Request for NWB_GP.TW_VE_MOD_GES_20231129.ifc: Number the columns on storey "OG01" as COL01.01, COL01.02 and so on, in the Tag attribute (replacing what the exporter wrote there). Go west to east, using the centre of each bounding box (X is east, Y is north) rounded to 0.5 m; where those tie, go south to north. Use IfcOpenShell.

First a look at what the model holds.

```python
import ifcopenshell
import ifcopenshell.util.element
import ifcopenshell.util.placement

model = ifcopenshell.open("NWB_GP.TW_VE_MOD_GES_20231129.ifc")
print(model.schema)
storey = next(s for s in model.by_type("IfcBuildingStorey") if s.Name == "OG01")
columns = [e for e in ifcopenshell.util.element.get_decomposition(storey) if e.is_a("IfcColumn")]
for e in sorted(columns, key=lambda e: e.id()):
    origin = ifcopenshell.util.placement.get_local_placement(e.ObjectPlacement)[:3, 3]
    print(e.id(), e.Tag, e.Name, origin.round(2) + 0.0, sep=" | ")
```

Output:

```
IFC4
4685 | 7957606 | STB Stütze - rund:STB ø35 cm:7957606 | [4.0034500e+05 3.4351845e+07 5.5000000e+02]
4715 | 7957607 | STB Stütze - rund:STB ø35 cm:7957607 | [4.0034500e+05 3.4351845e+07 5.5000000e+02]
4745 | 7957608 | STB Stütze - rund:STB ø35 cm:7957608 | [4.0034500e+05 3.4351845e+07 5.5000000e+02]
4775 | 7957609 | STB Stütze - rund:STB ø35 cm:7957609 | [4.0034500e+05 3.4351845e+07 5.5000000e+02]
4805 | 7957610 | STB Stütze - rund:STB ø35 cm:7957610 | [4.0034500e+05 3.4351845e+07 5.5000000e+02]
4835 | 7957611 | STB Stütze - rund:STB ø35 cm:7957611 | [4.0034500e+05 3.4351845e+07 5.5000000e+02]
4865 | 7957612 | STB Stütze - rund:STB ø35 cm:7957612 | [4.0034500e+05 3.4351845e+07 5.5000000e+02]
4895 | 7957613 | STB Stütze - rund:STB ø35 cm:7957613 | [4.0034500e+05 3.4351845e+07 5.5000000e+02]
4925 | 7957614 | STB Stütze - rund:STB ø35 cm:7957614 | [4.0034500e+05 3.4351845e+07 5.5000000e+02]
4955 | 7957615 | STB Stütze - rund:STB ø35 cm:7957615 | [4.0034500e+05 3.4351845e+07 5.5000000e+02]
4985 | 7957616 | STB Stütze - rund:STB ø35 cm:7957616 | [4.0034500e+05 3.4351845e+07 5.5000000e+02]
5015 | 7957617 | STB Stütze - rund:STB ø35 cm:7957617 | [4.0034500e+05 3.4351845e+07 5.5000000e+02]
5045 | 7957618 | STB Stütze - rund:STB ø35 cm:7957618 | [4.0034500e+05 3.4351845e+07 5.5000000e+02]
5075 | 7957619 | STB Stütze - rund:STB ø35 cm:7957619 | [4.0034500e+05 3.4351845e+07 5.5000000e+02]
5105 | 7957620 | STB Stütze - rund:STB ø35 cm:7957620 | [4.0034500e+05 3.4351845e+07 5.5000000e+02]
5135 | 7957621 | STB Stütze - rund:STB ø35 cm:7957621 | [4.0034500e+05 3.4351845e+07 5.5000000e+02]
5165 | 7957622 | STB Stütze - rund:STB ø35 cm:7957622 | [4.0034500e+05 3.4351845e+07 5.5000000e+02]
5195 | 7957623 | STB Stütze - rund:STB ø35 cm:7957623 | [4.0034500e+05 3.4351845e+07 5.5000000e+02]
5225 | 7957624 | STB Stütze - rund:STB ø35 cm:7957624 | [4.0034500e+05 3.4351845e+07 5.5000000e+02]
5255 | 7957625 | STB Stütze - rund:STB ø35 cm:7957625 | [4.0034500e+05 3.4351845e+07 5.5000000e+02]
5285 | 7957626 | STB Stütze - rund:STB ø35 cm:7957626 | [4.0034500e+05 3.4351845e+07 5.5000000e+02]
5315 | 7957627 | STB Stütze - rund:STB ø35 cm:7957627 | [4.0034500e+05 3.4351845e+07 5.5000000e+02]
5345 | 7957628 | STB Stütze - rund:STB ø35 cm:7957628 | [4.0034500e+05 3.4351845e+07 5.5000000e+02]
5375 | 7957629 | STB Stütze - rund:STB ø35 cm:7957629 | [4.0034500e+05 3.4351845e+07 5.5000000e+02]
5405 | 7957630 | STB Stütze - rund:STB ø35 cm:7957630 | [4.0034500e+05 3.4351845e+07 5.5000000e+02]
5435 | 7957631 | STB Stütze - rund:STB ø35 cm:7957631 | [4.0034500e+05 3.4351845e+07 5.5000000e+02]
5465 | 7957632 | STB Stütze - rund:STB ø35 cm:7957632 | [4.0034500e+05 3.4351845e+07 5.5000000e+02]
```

```python
import ifcopenshell
import ifcopenshell.geom
import ifcopenshell.util.element
import ifcopenshell.util.shape

model = ifcopenshell.open("NWB_GP.TW_VE_MOD_GES_20231129.ifc")
settings = ifcopenshell.geom.settings()
settings.set("use-world-coords", True)


def centre(element):
    shape = ifcopenshell.geom.create_shape(settings, element)
    return ifcopenshell.util.shape.get_bbox_centroid(shape.geometry)


storey = next(s for s in model.by_type("IfcBuildingStorey") if s.Name == "OG01")
columns = [e for e in ifcopenshell.util.element.get_decomposition(storey) if e.is_a("IfcColumn")]

# Insertion points can sit at a corner or the storey origin, so sort by the geometry (in metres).
centres = {e: centre(e) for e in columns}
columns.sort(key=lambda e: (round(centres[e][0] / 0.5), centres[e][1]))

for i, e in enumerate(columns, start=1):
    number = f"COL01.{i:02d}"
    e.Tag = number
    print(e.id(), number)

model.write("NWB_GP.TW_VE_MOD_GES_20231129_rev.ifc")
```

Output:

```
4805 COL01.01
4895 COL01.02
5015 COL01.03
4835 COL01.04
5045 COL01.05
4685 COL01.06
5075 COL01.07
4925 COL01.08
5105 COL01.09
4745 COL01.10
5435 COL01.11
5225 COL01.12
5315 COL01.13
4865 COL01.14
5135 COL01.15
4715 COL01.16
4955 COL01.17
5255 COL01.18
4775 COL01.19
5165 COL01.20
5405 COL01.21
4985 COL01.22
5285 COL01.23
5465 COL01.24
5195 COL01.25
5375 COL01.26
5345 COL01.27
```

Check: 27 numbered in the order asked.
